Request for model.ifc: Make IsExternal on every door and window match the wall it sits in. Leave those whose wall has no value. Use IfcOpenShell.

First a look at what the model holds.

```python
import ifcopenshell
import ifcopenshell.util.element

model = ifcopenshell.open("model.ifc")
print(model.schema)
seen = {}
for e in model.by_type("IfcDoor") + model.by_type("IfcWindow"):
    if not e.FillsVoids:
        continue
    host = e.FillsVoids[0].RelatingOpeningElement.VoidsElements[0].RelatingBuildingElement
    own = ifcopenshell.util.element.get_pset(e, f"Pset_{e.is_a()[3:].removesuffix('StandardCase')}Common", "IsExternal")
    wall = ifcopenshell.util.element.get_pset(host, "Pset_WallCommon", "IsExternal")
    seen[e.is_a(), own, wall] = seen.get((e.is_a(), own, wall), 0) + 1
for (cls, own, wall), count in sorted(seen.items(), key=str):
    print(count, cls, "IsExternal:", own, "| host wall:", wall)
```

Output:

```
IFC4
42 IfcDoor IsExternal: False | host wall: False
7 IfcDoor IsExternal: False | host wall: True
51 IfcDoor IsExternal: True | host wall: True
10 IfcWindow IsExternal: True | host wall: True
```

```python
import ifcopenshell
import ifcopenshell.api.pset
import ifcopenshell.util.element

model = ifcopenshell.open("model.ifc")

count = 0
for ifc_class, pset_name in (("IfcDoor", "Pset_DoorCommon"), ("IfcWindow", "Pset_WindowCommon")):
    for e in model.by_type(ifc_class):
        if not e.FillsVoids:
            continue
        host = e.FillsVoids[0].RelatingOpeningElement.VoidsElements[0].RelatingBuildingElement
        external = ifcopenshell.util.element.get_pset(host, "Pset_WallCommon", "IsExternal")
        if external is None or ifcopenshell.util.element.get_pset(e, pset_name, "IsExternal") == external:
            continue
        pset = ifcopenshell.api.pset.add_pset(model, product=e, name=pset_name)
        ifcopenshell.api.pset.edit_pset(model, pset=pset, properties={"IsExternal": external})
        count += 1

print(count, "updated")

model.write("model_rev.ifc")
```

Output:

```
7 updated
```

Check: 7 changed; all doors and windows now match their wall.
